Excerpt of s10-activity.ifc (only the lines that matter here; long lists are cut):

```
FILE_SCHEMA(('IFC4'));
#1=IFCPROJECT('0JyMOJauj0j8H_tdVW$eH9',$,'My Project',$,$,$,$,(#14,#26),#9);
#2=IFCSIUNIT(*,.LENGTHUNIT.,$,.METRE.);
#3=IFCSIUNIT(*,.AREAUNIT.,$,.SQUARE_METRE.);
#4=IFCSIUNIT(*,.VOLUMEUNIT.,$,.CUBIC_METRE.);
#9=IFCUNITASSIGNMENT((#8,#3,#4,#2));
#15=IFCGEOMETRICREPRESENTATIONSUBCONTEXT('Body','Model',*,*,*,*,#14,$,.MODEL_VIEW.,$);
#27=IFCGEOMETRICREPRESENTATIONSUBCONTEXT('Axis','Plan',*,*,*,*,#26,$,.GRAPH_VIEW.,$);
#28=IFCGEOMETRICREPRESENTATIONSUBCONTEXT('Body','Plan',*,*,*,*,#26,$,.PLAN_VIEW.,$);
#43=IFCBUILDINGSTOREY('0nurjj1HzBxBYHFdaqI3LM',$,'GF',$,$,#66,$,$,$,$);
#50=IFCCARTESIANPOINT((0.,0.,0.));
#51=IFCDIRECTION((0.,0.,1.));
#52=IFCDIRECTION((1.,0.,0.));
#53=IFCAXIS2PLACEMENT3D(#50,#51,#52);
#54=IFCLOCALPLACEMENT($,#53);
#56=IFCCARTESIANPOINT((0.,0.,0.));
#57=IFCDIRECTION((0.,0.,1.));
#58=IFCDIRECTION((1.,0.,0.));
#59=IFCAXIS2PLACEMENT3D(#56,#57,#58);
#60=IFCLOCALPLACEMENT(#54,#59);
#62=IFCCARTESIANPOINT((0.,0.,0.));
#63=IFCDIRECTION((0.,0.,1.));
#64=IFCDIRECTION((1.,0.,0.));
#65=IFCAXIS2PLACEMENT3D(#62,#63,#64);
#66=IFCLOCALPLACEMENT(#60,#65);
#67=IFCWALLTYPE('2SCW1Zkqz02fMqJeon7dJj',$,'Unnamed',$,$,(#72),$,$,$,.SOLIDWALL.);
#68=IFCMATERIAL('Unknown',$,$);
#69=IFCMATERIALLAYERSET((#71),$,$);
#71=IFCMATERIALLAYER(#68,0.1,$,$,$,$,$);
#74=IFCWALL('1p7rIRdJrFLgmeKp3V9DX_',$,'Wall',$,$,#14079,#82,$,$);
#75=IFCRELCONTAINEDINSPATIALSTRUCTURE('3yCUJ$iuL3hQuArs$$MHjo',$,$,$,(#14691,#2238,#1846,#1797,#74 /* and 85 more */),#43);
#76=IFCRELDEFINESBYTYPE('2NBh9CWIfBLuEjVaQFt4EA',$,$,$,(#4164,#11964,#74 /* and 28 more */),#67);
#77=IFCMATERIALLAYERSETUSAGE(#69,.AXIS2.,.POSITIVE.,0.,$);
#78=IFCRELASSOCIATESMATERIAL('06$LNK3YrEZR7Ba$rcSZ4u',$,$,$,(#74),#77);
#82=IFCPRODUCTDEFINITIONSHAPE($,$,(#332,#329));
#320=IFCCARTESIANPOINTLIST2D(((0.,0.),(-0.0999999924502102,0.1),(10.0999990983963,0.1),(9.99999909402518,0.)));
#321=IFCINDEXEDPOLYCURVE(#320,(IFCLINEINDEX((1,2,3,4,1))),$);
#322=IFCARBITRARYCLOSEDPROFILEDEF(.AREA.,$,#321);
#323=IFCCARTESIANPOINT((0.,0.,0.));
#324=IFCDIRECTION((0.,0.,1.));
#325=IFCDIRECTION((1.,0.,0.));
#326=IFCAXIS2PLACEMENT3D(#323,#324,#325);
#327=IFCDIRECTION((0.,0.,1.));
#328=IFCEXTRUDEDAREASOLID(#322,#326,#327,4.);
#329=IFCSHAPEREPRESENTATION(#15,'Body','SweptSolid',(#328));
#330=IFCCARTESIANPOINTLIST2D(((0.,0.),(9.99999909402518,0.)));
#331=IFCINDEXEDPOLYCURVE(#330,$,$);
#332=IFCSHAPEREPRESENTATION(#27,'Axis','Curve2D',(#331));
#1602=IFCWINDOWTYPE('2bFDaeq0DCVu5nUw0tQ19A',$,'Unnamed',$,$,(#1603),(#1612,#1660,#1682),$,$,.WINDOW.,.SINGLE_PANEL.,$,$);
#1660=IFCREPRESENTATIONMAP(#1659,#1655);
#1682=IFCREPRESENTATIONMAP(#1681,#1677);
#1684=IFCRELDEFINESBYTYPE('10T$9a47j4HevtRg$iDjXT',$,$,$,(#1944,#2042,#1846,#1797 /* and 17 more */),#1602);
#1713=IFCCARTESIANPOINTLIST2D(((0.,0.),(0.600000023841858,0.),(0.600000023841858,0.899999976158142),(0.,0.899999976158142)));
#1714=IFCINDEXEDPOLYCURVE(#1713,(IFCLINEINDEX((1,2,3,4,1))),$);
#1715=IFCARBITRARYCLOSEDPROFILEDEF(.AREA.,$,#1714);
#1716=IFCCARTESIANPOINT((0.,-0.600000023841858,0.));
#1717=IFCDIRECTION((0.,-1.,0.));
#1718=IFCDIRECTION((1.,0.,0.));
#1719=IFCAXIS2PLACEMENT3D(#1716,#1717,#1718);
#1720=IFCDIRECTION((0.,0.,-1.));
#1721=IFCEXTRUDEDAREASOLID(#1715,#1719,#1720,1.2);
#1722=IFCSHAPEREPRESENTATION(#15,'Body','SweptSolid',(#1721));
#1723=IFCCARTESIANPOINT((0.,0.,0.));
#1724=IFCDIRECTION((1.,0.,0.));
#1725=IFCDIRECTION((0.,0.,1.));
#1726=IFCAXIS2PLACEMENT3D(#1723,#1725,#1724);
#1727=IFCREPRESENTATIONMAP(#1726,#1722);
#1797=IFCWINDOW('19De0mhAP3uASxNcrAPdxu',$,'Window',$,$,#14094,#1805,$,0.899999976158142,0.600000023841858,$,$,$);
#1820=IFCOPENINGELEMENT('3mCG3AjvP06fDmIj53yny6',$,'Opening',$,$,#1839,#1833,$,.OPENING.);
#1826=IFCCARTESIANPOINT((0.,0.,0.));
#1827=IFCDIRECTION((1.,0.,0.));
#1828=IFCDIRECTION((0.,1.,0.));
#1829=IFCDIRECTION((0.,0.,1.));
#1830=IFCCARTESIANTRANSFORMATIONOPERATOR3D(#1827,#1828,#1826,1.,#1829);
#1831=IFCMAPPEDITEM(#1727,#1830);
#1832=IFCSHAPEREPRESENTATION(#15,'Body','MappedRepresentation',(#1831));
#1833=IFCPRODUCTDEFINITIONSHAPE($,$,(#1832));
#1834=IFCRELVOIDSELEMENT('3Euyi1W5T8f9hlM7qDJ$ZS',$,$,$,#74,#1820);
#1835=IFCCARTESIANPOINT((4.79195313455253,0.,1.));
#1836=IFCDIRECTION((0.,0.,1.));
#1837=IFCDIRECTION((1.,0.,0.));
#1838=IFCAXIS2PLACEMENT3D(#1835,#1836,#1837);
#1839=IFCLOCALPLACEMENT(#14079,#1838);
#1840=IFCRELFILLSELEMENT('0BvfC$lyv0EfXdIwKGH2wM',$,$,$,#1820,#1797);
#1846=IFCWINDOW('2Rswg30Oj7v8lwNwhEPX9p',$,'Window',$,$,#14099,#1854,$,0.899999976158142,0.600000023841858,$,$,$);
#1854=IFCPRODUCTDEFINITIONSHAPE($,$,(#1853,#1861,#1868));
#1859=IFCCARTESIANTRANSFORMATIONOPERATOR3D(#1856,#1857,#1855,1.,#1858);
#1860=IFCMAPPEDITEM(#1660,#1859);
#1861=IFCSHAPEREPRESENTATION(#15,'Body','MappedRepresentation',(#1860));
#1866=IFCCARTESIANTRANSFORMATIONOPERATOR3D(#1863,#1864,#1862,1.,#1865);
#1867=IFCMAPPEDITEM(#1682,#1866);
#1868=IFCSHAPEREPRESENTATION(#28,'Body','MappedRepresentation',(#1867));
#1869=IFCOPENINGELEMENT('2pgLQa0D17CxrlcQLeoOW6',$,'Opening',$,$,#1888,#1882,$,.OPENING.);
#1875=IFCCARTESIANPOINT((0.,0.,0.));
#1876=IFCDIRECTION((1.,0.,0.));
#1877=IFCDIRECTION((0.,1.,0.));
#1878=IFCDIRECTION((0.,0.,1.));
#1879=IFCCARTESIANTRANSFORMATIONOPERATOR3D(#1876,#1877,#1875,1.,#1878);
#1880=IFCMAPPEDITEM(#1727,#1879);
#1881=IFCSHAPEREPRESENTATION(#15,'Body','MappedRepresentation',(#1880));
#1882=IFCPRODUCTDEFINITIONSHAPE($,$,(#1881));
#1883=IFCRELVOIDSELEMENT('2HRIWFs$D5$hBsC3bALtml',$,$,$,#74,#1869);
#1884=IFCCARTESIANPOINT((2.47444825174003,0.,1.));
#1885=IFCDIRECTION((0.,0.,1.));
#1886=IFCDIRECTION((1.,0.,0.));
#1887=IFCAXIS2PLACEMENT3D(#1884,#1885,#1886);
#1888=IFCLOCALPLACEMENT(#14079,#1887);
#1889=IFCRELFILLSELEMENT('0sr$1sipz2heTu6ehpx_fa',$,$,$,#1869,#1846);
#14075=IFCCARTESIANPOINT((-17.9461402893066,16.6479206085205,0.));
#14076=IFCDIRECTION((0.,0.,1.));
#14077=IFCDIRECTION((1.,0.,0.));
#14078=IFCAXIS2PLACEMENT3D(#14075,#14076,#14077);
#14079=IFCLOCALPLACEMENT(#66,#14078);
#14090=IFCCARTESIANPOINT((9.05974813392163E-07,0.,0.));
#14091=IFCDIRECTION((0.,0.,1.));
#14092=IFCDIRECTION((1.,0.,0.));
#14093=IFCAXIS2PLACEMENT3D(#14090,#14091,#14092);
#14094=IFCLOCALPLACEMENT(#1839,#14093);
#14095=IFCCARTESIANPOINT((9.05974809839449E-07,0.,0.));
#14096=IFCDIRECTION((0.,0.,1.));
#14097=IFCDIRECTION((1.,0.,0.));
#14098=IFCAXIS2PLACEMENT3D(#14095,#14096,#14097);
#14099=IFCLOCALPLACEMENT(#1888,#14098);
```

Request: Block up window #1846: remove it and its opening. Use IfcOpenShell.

```python
import ifcopenshell
import ifcopenshell.api.feature
import ifcopenshell.api.root
import ifcopenshell.geom
import ifcopenshell.util.shape

model = ifcopenshell.open("s10-activity.ifc")
settings = ifcopenshell.geom.settings()


def volume(element):
    """Net volume in cubic metres, openings subtracted."""
    shape = ifcopenshell.geom.create_shape(settings, element)
    return ifcopenshell.util.shape.get_volume(shape.geometry)


window = model.by_guid("2Rswg30Oj7v8lwNwhEPX9p")
opening = window.FillsVoids[0].RelatingOpeningElement
wall = opening.VoidsElements[0].RelatingBuildingElement
before = volume(wall)

ifcopenshell.api.root.remove_product(model, product=window)
ifcopenshell.api.feature.remove_feature(model, feature=opening)

after = volume(wall)

print(f"wall volume {before:.3f} -> {after:.3f} m3")

model.write("s10-activity_edited.ifc")
```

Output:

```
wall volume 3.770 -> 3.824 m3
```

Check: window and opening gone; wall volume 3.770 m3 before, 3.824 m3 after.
